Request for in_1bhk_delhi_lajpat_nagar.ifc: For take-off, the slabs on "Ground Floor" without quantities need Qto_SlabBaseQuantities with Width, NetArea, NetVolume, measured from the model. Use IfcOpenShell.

First a look at what the model holds.

```python
import ifcopenshell
import ifcopenshell.util.element
import ifcopenshell.util.unit

model = ifcopenshell.open("in_1bhk_delhi_lajpat_nagar.ifc")
print(model.schema)
for unit_type in ("LENGTHUNIT", "AREAUNIT", "VOLUMEUNIT"):
    print(unit_type, ifcopenshell.util.unit.calculate_unit_scale(model, unit_type))
storey = next(s for s in model.by_type("IfcBuildingStorey") if s.Name == "Ground Floor")
slabs = [e for e in ifcopenshell.util.element.get_decomposition(storey) if e.is_a("IfcSlab")]
for e in sorted(slabs, key=lambda e: e.id()):
    print(e.id(), e.is_a(), e.Name, list(ifcopenshell.util.element.get_psets(e, qtos_only=True)), sep=" | ")
```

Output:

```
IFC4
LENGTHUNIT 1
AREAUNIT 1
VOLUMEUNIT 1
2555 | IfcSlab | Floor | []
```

```python
import ifcopenshell
import ifcopenshell.api.pset
import ifcopenshell.geom
import ifcopenshell.util.element
import ifcopenshell.util.shape
import ifcopenshell.util.unit

model = ifcopenshell.open("in_1bhk_delhi_lajpat_nagar.ifc")
unit_scale = ifcopenshell.util.unit.calculate_unit_scale(model)
area_scale = ifcopenshell.util.unit.calculate_unit_scale(model, "AREAUNIT")
volume_scale = ifcopenshell.util.unit.calculate_unit_scale(model, "VOLUMEUNIT")
settings = ifcopenshell.geom.settings()

storey = next(s for s in model.by_type("IfcBuildingStorey") if s.Name == "Ground Floor")
slabs = [e for e in ifcopenshell.util.element.get_decomposition(storey) if e.is_a("IfcSlab")]

for e in sorted(slabs, key=lambda e: e.id()):
    if ifcopenshell.util.element.get_psets(e, qtos_only=True, should_inherit=False):
        continue
    # Geometry comes back in metres, in the element's own axes.
    shape = ifcopenshell.geom.create_shape(settings, e)
    values = {
        "Width": ifcopenshell.util.shape.get_z(shape.geometry) / unit_scale,
        "NetArea": ifcopenshell.util.shape.get_footprint_area(shape.geometry) / area_scale,
        "NetVolume": ifcopenshell.util.shape.get_volume(shape.geometry) / volume_scale,
    }
    qto = ifcopenshell.api.pset.add_qto(model, product=e, name="Qto_SlabBaseQuantities")
    ifcopenshell.api.pset.edit_qto(model, qto=qto, properties=values)
    print(e.id(), {k: round(v, 3) for k, v in values.items()})

model.write("in_1bhk_delhi_lajpat_nagar-out.ifc")
```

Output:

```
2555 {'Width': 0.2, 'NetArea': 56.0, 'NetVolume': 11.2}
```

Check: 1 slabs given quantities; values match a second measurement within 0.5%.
